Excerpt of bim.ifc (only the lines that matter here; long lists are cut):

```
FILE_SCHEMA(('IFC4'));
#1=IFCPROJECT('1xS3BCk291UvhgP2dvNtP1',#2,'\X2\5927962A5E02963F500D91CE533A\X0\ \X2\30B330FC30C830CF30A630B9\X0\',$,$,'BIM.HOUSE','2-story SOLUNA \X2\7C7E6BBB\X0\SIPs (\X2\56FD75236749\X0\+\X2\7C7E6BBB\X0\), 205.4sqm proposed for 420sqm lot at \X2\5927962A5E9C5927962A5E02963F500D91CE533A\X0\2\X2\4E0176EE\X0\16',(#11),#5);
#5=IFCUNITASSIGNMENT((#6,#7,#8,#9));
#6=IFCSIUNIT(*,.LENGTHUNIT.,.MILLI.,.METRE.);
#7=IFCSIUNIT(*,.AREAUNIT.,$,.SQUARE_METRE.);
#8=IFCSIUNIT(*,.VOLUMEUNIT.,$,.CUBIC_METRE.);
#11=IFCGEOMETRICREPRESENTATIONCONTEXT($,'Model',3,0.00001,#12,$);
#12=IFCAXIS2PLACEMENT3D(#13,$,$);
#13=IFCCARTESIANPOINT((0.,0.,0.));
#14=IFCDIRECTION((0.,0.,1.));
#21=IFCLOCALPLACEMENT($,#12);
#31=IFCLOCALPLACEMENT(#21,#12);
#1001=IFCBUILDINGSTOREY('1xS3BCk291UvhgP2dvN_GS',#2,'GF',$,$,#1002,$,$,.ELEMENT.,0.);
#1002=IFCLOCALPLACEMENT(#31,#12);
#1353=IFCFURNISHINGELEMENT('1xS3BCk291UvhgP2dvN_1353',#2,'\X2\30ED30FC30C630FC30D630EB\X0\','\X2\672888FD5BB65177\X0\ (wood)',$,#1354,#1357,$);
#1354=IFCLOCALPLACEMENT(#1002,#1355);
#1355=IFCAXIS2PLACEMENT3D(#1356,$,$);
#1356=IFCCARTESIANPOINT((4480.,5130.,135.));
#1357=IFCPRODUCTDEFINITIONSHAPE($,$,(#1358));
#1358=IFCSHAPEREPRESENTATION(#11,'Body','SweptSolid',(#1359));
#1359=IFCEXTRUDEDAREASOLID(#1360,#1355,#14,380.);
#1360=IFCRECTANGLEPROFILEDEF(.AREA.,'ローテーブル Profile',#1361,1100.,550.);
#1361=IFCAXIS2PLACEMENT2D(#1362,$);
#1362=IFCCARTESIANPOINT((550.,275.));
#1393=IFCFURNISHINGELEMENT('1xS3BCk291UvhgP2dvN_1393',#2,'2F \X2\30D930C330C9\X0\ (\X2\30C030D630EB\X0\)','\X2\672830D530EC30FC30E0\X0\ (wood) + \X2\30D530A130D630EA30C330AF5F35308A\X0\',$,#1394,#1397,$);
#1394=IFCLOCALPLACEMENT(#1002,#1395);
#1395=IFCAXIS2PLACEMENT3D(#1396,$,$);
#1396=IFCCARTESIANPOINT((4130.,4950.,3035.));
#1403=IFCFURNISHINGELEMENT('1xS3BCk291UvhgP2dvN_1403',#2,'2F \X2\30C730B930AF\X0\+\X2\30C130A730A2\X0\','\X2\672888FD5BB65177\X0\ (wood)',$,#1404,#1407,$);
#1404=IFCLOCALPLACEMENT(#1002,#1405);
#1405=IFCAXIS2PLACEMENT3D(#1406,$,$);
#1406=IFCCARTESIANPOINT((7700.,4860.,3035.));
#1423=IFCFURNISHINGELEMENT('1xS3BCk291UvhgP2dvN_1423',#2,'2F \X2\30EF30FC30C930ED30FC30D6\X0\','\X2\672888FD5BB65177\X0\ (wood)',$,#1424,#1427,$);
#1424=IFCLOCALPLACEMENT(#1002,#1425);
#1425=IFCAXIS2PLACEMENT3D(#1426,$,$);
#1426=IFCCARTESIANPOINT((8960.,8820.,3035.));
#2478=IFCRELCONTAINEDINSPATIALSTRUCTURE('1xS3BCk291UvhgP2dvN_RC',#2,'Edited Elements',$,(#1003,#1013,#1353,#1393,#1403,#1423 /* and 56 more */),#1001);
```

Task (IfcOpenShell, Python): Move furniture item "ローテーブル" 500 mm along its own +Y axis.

```python
import ifcopenshell
import ifcopenshell.api.geometry
import ifcopenshell.util.placement
import ifcopenshell.util.unit

model = ifcopenshell.open("bim.ifc")
unit_scale = ifcopenshell.util.unit.calculate_unit_scale(model)

item = model.by_id(1353)
matrix = ifcopenshell.util.placement.get_local_placement(item.ObjectPlacement)
matrix[:3, 3] += matrix[:3, 1] * 0.5 / unit_scale
ifcopenshell.api.geometry.edit_object_placement(model, product=item, matrix=matrix, is_si=False)

print(ifcopenshell.util.placement.get_local_placement(item.ObjectPlacement).round(3) + 0.0)

model.write("bim_updated.ifc")
```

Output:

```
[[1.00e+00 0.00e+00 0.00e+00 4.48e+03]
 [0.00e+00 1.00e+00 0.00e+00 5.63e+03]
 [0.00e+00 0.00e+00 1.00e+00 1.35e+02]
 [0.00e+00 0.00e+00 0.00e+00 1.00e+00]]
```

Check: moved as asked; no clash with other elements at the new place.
